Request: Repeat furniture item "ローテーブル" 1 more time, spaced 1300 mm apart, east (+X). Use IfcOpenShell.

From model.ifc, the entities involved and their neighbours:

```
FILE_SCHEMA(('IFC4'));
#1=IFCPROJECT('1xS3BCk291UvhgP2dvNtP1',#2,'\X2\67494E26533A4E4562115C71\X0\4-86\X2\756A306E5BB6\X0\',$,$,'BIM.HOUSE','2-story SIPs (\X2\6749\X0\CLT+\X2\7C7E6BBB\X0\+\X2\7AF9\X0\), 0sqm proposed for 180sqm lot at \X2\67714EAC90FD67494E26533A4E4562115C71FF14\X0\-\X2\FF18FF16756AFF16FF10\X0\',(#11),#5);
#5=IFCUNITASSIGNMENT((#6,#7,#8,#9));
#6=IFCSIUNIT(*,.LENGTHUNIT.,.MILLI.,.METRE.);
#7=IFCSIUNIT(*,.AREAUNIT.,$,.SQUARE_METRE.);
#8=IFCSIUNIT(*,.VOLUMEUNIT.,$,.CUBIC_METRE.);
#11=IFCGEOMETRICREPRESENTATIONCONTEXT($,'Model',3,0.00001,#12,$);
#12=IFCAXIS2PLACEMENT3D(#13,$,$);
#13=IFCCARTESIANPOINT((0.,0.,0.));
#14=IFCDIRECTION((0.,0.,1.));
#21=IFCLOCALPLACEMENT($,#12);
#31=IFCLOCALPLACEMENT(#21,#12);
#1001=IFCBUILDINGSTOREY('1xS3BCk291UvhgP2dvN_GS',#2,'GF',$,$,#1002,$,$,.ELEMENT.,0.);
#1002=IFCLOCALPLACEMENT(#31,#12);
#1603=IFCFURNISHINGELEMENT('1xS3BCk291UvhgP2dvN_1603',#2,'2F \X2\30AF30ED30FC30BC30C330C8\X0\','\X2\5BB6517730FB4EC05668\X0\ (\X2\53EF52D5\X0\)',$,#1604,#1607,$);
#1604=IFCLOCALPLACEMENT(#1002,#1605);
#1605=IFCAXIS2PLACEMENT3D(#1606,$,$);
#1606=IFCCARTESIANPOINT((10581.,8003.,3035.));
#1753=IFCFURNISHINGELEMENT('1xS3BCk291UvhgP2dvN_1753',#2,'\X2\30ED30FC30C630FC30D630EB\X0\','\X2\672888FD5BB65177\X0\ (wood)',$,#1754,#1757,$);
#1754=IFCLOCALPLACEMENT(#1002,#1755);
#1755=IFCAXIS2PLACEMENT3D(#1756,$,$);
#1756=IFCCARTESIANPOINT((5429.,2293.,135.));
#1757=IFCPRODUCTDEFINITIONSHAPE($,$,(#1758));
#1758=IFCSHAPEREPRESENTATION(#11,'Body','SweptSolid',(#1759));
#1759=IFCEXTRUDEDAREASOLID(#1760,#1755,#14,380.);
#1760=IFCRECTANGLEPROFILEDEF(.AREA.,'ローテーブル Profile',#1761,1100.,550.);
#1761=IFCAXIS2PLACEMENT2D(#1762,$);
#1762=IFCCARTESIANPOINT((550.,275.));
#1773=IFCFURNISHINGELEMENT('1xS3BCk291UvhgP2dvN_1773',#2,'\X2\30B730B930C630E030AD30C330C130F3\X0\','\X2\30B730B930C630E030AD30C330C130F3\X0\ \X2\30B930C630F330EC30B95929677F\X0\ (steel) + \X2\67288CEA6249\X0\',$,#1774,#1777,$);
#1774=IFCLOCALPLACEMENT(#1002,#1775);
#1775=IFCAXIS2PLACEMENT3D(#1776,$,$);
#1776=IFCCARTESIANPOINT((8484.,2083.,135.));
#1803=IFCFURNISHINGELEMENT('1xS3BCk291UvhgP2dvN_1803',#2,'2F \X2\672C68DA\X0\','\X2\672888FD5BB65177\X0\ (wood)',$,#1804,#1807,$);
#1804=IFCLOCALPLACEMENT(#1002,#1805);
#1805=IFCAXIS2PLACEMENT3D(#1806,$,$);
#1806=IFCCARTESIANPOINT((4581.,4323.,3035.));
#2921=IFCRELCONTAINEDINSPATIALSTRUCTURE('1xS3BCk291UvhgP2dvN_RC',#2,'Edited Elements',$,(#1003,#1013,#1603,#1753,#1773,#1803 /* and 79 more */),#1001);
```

```python
import numpy as np
import ifcopenshell
import ifcopenshell.api.geometry
import ifcopenshell.api.root
import ifcopenshell.util.element
import ifcopenshell.util.placement

model = ifcopenshell.open("model.ifc")


def reuse_history(source, copy):
    """copy_class also copies each property set's owner history, people and application; keep the originals."""
    for rel in copy.IsDefinedBy:
        if rel.is_a("IfcRelDefinesByProperties") and (history := rel.RelatingPropertyDefinition.OwnerHistory):
            rel.RelatingPropertyDefinition.OwnerHistory = source.OwnerHistory
            ifcopenshell.util.element.remove_deep2(model, history)


source = model.by_id(1753)
base = ifcopenshell.util.placement.get_local_placement(source.ObjectPlacement)
step = np.array([1.0, 0.0, 0.0]) * 1300.0

for i in range(1, 2):
    copy = ifcopenshell.api.root.copy_class(model, product=source)
    copy.Representation = ifcopenshell.util.element.copy_deep(
        model, source.Representation, exclude=["IfcGeometricRepresentationContext", "IfcRepresentationMap"]
    )
    reuse_history(source, copy)
    matrix = base.copy()
    matrix[:3, 3] += i * step
    print("added at", matrix[:3, 3].round(3) + 0.0)
    ifcopenshell.api.geometry.edit_object_placement(model, product=copy, matrix=matrix, is_si=False)

model.write("model_v2.ifc")
```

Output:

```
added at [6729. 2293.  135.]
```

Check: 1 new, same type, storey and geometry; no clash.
